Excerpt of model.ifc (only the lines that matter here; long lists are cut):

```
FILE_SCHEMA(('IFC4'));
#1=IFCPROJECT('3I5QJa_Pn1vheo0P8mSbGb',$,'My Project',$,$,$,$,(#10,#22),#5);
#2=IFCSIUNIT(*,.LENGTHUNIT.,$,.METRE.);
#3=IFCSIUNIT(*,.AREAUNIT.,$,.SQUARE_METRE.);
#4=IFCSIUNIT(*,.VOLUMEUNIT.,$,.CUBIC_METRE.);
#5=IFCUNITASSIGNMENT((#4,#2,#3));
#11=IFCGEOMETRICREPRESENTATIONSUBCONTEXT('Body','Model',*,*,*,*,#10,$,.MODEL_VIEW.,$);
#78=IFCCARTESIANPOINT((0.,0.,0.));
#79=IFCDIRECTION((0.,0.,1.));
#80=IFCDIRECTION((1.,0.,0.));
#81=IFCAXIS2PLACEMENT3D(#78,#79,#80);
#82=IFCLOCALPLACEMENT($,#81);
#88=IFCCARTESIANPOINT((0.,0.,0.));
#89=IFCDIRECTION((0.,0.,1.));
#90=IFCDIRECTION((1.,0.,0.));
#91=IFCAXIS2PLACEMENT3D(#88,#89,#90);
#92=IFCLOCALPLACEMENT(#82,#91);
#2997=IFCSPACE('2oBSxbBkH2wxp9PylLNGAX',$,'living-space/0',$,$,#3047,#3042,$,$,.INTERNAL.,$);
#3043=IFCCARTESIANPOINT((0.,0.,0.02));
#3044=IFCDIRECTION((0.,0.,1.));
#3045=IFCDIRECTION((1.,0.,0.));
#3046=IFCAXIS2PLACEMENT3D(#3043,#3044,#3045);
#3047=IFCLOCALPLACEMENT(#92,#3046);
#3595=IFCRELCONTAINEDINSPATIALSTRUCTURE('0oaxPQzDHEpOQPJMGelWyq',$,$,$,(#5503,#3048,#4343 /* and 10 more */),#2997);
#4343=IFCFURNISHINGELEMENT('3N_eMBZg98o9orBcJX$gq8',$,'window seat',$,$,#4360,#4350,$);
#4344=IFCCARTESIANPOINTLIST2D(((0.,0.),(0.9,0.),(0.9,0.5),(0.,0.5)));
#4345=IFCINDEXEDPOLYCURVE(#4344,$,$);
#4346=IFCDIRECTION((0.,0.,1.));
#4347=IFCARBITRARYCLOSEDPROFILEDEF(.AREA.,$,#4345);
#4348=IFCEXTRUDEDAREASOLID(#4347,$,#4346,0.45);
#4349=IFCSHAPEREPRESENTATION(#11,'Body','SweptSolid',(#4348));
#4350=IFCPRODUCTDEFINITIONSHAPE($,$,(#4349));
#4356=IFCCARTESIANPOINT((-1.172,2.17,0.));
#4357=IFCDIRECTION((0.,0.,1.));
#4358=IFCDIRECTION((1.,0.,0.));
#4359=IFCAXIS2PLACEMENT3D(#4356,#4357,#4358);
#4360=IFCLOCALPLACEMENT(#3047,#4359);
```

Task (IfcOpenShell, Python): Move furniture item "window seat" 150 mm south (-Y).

```python
import ifcopenshell
import ifcopenshell.api.geometry
import ifcopenshell.util.placement
import ifcopenshell.util.unit

model = ifcopenshell.open("model.ifc")
unit_scale = ifcopenshell.util.unit.calculate_unit_scale(model)

item = model.by_guid("3N_eMBZg98o9orBcJX$gq8")
matrix = ifcopenshell.util.placement.get_local_placement(item.ObjectPlacement)
matrix[1, 3] -= 0.15 / unit_scale
ifcopenshell.api.geometry.edit_object_placement(model, product=item, matrix=matrix, is_si=False)

print(ifcopenshell.util.placement.get_local_placement(item.ObjectPlacement).round(3) + 0.0)

model.write("model_updated.ifc")
```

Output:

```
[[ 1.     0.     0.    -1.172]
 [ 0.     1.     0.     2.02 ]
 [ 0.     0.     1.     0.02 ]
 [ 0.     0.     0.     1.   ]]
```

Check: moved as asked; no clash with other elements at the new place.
